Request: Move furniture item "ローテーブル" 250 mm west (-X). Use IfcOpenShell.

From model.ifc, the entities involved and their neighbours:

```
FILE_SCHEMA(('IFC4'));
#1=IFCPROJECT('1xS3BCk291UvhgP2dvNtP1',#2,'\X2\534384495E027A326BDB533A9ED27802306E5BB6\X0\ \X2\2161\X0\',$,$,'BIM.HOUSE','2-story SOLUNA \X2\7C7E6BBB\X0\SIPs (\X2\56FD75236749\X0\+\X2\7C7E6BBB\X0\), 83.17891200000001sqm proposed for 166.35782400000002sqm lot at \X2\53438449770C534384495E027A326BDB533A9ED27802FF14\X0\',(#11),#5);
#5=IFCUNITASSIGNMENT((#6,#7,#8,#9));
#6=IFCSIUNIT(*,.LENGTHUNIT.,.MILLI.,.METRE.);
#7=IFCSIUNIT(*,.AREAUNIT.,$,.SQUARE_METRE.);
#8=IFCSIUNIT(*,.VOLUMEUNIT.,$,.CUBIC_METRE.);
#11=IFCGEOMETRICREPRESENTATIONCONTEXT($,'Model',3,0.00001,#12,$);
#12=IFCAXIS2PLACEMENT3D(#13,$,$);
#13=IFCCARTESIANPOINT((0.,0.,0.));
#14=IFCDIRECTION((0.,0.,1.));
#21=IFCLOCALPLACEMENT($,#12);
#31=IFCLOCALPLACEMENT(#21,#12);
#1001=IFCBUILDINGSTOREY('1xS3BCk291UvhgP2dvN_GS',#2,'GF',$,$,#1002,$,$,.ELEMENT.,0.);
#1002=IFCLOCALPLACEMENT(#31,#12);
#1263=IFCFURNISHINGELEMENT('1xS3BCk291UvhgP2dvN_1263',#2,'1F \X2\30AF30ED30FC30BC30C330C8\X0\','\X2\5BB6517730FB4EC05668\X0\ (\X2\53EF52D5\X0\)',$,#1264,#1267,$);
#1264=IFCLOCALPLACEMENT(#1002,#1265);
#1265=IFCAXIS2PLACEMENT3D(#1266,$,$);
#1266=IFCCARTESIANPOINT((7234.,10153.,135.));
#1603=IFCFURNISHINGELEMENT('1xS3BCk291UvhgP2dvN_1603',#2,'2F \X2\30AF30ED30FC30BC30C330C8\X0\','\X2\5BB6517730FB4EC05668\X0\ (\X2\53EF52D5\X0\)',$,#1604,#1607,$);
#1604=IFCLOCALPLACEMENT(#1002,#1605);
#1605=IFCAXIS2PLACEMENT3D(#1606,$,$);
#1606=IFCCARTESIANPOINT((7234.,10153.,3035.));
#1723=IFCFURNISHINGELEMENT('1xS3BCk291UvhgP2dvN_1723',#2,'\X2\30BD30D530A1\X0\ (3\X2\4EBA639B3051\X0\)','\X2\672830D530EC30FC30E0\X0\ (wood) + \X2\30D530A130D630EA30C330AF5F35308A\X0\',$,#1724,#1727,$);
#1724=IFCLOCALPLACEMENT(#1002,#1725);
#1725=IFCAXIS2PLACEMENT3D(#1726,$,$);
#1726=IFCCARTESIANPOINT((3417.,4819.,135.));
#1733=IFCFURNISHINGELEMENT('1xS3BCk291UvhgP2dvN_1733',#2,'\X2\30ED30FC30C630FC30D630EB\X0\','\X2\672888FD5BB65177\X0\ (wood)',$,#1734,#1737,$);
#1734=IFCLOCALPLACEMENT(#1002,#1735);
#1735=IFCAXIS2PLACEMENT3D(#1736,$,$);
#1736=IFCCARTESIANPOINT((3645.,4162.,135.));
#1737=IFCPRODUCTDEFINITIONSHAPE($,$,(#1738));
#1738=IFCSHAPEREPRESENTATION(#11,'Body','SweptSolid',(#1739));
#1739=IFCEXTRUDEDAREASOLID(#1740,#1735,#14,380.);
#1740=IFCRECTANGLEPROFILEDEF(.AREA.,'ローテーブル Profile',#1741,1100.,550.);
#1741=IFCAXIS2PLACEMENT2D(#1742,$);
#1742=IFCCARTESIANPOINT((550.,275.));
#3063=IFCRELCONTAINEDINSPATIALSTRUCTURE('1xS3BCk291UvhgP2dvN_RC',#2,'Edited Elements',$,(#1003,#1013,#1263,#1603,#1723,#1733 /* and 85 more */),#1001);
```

```python
import ifcopenshell
import ifcopenshell.api.geometry
import ifcopenshell.util.placement
import ifcopenshell.util.unit

model = ifcopenshell.open("model.ifc")
unit_scale = ifcopenshell.util.unit.calculate_unit_scale(model)

item = model.by_id(1733)
matrix = ifcopenshell.util.placement.get_local_placement(item.ObjectPlacement)
matrix[0, 3] -= 0.25 / unit_scale
ifcopenshell.api.geometry.edit_object_placement(model, product=item, matrix=matrix, is_si=False)

print(ifcopenshell.util.placement.get_local_placement(item.ObjectPlacement).round(3) + 0.0)

model.write("model_rev.ifc")
```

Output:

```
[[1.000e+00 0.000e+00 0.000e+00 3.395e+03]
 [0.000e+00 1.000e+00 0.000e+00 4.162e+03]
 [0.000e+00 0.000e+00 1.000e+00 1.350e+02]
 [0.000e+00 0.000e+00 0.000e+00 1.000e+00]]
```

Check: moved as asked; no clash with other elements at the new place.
